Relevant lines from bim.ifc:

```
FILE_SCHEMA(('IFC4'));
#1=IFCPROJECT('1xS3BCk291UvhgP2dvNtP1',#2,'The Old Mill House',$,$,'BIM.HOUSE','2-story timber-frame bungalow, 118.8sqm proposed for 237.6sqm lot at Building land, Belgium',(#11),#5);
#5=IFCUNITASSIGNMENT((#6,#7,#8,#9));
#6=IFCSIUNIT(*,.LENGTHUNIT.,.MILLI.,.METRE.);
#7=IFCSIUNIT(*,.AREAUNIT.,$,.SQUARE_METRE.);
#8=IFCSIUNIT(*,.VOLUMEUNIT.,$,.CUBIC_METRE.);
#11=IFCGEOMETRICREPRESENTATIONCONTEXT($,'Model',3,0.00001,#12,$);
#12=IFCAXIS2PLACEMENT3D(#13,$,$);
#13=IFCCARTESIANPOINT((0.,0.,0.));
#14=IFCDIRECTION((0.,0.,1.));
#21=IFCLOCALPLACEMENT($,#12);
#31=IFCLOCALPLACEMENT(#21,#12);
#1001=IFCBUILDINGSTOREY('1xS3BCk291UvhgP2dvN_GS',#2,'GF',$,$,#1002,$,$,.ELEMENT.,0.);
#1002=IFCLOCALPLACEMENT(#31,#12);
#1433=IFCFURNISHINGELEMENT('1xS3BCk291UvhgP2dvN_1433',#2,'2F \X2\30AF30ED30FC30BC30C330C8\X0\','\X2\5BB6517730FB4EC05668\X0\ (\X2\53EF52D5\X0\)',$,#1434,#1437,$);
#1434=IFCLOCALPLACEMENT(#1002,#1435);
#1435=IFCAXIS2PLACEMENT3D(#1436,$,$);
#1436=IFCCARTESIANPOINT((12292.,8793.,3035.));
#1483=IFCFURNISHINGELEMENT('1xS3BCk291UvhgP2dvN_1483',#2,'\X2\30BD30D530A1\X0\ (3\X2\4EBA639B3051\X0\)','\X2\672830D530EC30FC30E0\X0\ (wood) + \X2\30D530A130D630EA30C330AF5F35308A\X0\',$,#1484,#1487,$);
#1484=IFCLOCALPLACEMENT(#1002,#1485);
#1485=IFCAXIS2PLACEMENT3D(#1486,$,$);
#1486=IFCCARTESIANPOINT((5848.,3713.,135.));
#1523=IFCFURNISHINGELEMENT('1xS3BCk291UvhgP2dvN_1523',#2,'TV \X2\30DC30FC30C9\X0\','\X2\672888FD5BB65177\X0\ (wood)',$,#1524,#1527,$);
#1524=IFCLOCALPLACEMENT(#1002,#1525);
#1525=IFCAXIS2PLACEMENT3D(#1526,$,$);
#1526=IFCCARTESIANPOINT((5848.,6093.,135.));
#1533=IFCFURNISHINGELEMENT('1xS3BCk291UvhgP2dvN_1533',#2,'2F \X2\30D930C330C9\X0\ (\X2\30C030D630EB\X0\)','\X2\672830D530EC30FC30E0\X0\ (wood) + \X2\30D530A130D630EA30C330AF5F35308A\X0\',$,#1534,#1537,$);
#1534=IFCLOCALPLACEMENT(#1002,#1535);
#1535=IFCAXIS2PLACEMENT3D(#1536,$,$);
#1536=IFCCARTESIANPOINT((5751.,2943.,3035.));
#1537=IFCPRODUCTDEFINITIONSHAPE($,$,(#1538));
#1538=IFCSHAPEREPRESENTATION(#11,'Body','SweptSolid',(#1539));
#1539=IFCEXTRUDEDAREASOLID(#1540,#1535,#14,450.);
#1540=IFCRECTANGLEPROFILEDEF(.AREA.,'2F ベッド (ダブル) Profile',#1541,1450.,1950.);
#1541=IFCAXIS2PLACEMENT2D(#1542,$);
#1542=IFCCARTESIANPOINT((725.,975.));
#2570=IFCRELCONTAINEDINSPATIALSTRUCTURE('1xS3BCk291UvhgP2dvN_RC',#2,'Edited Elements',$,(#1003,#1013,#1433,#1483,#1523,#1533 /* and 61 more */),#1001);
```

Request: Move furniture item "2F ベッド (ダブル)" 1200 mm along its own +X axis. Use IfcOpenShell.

```python
import ifcopenshell
import ifcopenshell.api.geometry
import ifcopenshell.util.placement

model = ifcopenshell.open("bim.ifc")

item = model.by_id(1533)
matrix = ifcopenshell.util.placement.get_local_placement(item.ObjectPlacement)
matrix[:3, 3] += matrix[:3, 0] * 1200.0
ifcopenshell.api.geometry.edit_object_placement(model, product=item, matrix=matrix, is_si=False)

print(ifcopenshell.util.placement.get_local_placement(item.ObjectPlacement).round(3) + 0.0)

model.write("bim-out.ifc")
```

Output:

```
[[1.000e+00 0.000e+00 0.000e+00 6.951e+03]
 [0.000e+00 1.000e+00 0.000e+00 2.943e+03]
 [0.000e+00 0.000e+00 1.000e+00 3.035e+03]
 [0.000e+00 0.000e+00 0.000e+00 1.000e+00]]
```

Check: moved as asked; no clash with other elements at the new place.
